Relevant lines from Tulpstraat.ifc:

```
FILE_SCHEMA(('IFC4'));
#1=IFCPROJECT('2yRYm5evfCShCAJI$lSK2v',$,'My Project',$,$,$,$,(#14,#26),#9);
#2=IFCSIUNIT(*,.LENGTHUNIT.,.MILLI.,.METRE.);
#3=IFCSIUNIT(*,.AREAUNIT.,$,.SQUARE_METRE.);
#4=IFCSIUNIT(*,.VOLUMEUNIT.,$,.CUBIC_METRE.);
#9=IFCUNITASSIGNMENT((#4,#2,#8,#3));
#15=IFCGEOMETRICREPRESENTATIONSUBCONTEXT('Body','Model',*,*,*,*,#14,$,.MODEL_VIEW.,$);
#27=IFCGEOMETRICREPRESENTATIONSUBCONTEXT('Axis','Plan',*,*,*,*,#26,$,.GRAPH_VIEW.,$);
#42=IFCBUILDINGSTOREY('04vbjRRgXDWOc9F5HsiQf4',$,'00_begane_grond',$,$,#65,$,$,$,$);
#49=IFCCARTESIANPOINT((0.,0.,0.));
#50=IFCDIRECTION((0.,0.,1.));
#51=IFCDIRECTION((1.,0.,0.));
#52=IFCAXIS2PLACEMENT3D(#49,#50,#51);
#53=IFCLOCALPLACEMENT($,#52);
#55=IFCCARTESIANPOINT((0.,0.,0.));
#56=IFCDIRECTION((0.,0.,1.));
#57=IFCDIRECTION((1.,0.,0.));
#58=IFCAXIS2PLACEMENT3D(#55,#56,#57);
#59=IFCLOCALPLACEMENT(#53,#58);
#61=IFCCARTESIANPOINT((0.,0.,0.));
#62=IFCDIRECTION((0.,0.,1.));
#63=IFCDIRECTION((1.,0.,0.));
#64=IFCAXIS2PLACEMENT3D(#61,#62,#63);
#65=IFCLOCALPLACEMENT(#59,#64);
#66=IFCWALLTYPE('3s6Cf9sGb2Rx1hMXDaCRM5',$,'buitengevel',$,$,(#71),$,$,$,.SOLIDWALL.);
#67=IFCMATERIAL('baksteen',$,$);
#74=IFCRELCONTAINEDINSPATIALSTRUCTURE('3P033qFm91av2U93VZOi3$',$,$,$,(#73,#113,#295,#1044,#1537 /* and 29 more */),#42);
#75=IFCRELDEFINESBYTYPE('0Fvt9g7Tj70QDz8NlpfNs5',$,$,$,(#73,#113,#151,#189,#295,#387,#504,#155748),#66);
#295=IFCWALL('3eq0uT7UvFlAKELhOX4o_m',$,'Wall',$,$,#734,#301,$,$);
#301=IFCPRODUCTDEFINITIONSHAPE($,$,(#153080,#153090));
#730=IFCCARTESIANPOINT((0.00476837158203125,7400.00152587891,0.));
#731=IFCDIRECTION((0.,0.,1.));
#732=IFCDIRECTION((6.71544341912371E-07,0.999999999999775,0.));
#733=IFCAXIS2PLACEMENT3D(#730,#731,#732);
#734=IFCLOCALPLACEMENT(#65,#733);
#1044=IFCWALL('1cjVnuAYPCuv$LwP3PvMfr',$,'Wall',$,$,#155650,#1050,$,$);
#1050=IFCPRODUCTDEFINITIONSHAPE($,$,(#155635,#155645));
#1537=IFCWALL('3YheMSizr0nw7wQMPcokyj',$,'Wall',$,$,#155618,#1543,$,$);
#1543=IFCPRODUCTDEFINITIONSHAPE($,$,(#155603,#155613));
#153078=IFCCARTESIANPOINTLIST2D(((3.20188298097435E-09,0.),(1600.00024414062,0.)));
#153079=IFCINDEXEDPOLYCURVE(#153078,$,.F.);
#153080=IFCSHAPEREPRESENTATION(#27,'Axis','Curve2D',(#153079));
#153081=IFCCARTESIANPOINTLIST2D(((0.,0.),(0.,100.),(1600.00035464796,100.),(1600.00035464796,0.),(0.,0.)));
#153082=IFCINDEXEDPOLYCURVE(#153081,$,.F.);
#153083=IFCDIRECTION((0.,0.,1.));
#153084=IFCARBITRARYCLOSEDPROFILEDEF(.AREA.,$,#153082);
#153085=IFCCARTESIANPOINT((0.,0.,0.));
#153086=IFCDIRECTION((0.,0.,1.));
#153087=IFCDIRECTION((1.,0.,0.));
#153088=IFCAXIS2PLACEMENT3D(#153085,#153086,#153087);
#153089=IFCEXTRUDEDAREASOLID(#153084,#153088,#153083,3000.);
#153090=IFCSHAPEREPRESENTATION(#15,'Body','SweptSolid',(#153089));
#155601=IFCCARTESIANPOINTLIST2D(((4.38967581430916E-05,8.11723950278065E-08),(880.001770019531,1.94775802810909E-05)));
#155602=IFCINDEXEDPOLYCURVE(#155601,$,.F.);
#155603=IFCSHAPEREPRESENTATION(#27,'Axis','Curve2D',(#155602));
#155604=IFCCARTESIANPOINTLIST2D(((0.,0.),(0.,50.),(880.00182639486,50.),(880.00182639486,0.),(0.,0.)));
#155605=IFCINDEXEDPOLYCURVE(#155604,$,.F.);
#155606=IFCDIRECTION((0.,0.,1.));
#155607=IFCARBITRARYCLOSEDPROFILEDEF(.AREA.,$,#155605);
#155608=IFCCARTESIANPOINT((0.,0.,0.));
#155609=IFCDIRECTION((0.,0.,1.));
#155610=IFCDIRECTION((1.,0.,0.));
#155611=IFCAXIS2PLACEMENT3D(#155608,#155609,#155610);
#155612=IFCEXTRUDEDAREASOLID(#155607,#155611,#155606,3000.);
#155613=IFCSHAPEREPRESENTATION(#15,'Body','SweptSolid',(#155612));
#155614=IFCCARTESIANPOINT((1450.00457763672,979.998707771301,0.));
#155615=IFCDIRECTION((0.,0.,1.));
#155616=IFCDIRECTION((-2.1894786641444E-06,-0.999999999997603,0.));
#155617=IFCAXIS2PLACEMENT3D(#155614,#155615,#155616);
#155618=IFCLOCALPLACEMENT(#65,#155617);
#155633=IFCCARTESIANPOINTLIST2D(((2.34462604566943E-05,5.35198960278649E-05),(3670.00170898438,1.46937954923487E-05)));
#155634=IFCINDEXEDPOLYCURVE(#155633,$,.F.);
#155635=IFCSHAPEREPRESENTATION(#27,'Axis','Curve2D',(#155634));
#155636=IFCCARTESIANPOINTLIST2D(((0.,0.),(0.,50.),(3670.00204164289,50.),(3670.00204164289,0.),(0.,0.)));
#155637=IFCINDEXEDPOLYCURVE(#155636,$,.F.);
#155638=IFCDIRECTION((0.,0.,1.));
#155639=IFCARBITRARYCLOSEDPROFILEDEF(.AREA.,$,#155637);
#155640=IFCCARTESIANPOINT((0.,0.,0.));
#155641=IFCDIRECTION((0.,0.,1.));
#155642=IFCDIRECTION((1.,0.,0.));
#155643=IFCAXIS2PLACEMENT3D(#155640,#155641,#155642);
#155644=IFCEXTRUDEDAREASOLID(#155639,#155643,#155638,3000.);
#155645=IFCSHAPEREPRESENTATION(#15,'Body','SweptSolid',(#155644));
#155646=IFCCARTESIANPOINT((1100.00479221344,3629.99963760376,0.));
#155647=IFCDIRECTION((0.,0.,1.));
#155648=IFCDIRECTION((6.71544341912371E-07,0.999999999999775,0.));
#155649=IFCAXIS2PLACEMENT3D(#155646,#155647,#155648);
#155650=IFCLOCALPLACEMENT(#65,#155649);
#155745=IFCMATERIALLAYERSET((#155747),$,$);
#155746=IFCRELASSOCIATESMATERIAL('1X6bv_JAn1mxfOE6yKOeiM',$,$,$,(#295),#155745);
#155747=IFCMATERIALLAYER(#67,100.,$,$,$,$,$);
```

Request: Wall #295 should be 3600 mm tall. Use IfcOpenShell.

```python
import ifcopenshell
import ifcopenshell.geom
import ifcopenshell.util.representation
import ifcopenshell.util.shape
import ifcopenshell.util.unit

model = ifcopenshell.open("Tulpstraat.ifc")
unit_scale = ifcopenshell.util.unit.calculate_unit_scale(model)
settings = ifcopenshell.geom.settings()


def volume(element):
    """Net volume in cubic metres, openings subtracted."""
    shape = ifcopenshell.geom.create_shape(settings, element)
    return ifcopenshell.util.shape.get_volume(shape.geometry)


wall = model.by_id(295)
before = volume(wall)

body = ifcopenshell.util.representation.get_representation(wall, "Model", "Body")
solid = body.Items[0]
old_height = solid.Depth
solid.Depth = 3.6 / unit_scale
after = volume(wall)

print(f"height {old_height:g} -> {solid.Depth:g}, volume {before:.3f} -> {after:.3f} m3")

model.write("Tulpstraat-out.ifc")
```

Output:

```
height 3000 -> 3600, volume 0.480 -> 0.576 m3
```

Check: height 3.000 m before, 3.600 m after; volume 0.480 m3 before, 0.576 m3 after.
